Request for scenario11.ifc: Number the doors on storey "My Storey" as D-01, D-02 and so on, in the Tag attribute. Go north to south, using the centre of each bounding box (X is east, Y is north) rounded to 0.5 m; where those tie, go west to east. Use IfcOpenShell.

First a look at what the model holds.

```python
import ifcopenshell
import ifcopenshell.util.element
import ifcopenshell.util.placement

model = ifcopenshell.open("scenario11.ifc")
print(model.schema)
storey = next(s for s in model.by_type("IfcBuildingStorey") if s.Name == "My Storey")
doors = [e for e in ifcopenshell.util.element.get_decomposition(storey) if e.is_a("IfcDoor")]
for e in sorted(doors, key=lambda e: e.id()):
    origin = ifcopenshell.util.placement.get_local_placement(e.ObjectPlacement)[:3, 3]
    print(e.id(), e.Tag, e.Name, origin.round(2) + 0.0, sep=" | ")
```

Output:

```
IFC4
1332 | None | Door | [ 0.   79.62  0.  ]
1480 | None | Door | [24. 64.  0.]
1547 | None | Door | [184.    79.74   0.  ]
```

```python
import ifcopenshell
import ifcopenshell.geom
import ifcopenshell.util.element
import ifcopenshell.util.shape

model = ifcopenshell.open("scenario11.ifc")
settings = ifcopenshell.geom.settings()
settings.set("use-world-coords", True)


def centre(element):
    shape = ifcopenshell.geom.create_shape(settings, element)
    return ifcopenshell.util.shape.get_bbox_centroid(shape.geometry)


storey = next(s for s in model.by_type("IfcBuildingStorey") if s.Name == "My Storey")
doors = [e for e in ifcopenshell.util.element.get_decomposition(storey) if e.is_a("IfcDoor")]

# Insertion points can sit at a corner or the storey origin, so sort by the geometry (in metres).
centres = {e: centre(e) for e in doors}
doors.sort(key=lambda e: (-round(centres[e][1] / 0.5), centres[e][0]))

for i, e in enumerate(doors, start=1):
    number = f"D-{i:02d}"
    e.Tag = number
    print(e.id(), number)

model.write("scenario11-out.ifc")
```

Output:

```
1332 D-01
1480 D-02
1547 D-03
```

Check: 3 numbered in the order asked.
